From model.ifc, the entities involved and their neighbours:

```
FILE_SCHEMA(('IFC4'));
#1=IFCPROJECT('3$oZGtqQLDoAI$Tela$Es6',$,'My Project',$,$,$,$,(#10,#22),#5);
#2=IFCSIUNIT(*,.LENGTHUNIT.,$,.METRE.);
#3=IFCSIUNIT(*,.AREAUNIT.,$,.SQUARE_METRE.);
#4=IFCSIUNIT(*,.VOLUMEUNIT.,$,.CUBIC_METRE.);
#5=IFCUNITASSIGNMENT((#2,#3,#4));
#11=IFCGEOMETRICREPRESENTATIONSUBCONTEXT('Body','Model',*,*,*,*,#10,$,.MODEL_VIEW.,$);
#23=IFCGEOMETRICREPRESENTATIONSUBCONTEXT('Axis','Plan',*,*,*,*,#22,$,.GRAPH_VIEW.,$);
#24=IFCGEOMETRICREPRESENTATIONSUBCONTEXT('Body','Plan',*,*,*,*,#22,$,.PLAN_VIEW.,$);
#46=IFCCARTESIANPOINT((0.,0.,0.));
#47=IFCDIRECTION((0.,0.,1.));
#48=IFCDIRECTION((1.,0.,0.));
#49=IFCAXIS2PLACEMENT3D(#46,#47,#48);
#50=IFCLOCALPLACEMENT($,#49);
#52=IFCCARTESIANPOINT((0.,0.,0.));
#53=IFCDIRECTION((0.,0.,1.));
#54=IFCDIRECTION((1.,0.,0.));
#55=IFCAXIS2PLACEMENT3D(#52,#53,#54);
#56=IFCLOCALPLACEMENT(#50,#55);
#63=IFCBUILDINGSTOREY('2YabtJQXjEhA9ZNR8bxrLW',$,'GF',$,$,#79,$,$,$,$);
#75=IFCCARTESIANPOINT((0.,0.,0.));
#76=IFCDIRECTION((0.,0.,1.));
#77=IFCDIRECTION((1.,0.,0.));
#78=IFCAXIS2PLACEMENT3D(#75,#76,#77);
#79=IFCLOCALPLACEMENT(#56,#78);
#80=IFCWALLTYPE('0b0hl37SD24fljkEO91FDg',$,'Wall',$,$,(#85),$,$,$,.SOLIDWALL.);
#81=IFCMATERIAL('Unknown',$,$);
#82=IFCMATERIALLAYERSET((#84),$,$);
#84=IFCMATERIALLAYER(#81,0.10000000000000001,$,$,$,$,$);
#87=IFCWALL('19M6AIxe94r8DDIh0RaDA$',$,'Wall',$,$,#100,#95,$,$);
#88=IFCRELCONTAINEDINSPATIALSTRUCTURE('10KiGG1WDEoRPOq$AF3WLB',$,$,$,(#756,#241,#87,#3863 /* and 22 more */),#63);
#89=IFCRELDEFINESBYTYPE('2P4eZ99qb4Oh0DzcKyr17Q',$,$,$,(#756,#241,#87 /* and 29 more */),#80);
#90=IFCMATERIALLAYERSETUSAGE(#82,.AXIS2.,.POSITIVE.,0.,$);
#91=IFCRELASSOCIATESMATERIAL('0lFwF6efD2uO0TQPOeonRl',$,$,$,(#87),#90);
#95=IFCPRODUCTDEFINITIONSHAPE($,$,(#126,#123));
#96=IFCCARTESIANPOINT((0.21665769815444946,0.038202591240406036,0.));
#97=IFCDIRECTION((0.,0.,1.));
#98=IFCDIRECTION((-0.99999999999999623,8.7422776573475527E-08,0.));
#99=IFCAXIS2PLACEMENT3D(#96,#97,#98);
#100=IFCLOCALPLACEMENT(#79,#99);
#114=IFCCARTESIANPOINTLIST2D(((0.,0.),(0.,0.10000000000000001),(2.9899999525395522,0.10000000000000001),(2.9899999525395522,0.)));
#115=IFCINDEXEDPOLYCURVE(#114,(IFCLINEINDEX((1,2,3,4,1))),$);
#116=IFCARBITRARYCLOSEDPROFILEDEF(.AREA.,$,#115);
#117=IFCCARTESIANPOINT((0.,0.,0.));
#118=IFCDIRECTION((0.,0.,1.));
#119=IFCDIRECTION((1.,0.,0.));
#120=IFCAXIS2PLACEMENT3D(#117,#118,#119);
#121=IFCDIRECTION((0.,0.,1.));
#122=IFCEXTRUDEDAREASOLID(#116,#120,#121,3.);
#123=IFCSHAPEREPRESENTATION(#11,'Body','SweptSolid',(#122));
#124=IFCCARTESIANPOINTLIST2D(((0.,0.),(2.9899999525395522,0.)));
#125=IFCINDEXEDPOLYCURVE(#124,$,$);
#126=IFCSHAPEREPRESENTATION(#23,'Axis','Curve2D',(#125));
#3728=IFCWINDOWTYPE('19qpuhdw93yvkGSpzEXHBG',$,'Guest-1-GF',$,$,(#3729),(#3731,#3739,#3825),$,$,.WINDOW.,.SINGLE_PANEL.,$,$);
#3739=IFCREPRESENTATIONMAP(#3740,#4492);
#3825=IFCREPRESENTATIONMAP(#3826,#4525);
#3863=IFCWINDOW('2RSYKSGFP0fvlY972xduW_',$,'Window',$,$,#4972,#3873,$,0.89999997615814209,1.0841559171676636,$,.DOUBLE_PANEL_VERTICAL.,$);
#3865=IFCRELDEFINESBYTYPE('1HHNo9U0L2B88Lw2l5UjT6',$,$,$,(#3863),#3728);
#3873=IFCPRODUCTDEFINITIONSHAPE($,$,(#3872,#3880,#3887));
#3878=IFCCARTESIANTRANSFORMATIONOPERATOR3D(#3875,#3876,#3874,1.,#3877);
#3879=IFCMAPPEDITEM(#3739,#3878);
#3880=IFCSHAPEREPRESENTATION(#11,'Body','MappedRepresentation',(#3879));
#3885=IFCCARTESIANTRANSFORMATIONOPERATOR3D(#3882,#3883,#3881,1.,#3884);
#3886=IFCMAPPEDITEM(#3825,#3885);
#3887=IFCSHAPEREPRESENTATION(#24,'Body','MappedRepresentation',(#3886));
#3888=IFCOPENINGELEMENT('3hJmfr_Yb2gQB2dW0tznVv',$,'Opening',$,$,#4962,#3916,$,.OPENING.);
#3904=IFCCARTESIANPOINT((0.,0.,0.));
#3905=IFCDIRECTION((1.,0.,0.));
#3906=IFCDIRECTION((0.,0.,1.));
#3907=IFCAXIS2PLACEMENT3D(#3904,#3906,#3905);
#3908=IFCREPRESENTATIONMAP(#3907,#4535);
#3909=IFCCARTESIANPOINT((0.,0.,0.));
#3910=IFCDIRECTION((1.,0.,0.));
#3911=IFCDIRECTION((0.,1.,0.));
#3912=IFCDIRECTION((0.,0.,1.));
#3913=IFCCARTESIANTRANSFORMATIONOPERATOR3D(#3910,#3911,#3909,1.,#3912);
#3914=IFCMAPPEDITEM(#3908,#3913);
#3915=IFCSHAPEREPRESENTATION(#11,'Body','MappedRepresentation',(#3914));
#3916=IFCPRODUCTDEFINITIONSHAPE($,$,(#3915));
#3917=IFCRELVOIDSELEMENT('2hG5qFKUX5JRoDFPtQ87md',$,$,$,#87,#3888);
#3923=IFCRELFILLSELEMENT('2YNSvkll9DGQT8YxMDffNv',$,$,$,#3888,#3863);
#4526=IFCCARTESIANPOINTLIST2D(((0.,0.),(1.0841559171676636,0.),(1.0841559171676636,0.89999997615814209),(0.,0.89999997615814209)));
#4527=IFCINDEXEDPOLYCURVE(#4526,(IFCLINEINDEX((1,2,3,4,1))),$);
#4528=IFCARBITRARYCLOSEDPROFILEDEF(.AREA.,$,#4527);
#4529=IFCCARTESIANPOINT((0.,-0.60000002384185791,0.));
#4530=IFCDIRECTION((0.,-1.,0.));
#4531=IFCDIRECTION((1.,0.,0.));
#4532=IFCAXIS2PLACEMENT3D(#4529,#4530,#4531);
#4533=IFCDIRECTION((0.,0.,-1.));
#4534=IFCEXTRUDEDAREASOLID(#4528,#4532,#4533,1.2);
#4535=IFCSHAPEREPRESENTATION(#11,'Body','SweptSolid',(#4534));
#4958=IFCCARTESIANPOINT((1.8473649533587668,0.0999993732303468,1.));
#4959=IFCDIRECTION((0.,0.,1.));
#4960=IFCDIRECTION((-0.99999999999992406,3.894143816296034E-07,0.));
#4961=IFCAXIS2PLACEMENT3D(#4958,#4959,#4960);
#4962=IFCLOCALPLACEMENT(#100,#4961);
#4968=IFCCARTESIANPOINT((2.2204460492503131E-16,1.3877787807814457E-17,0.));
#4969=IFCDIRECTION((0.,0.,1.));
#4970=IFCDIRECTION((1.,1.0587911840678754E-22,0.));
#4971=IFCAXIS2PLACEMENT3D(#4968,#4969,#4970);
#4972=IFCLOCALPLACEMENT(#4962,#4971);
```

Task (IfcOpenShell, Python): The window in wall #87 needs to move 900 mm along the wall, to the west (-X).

```python
import ifcopenshell
import ifcopenshell.api.geometry
import ifcopenshell.util.placement
import ifcopenshell.util.unit

model = ifcopenshell.open("model.ifc")
unit_scale = ifcopenshell.util.unit.calculate_unit_scale(model)

window = model.by_id(3863)
opening = window.FillsVoids[0].RelatingOpeningElement
wall = opening.VoidsElements[0].RelatingBuildingElement

wall_matrix = ifcopenshell.util.placement.get_local_placement(wall.ObjectPlacement)
shift = wall_matrix[:3, 0] * 0.9 / unit_scale
before = ifcopenshell.util.placement.get_local_placement(window.ObjectPlacement)[:3, 3].copy()

# The window is placed relative to its opening, so it follows when the opening moves.
matrix = ifcopenshell.util.placement.get_local_placement(opening.ObjectPlacement)
matrix[:3, 3] += shift
ifcopenshell.api.geometry.edit_object_placement(
    model, product=opening, matrix=matrix, is_si=False, should_transform_children=True
)

after = ifcopenshell.util.placement.get_local_placement(window.ObjectPlacement)[:3, 3]
print("window moved by", (after - before).round(3) + 0.0)

model.write("model_updated.ifc")
```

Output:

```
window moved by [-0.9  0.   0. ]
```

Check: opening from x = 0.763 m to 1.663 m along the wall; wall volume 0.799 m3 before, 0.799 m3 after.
